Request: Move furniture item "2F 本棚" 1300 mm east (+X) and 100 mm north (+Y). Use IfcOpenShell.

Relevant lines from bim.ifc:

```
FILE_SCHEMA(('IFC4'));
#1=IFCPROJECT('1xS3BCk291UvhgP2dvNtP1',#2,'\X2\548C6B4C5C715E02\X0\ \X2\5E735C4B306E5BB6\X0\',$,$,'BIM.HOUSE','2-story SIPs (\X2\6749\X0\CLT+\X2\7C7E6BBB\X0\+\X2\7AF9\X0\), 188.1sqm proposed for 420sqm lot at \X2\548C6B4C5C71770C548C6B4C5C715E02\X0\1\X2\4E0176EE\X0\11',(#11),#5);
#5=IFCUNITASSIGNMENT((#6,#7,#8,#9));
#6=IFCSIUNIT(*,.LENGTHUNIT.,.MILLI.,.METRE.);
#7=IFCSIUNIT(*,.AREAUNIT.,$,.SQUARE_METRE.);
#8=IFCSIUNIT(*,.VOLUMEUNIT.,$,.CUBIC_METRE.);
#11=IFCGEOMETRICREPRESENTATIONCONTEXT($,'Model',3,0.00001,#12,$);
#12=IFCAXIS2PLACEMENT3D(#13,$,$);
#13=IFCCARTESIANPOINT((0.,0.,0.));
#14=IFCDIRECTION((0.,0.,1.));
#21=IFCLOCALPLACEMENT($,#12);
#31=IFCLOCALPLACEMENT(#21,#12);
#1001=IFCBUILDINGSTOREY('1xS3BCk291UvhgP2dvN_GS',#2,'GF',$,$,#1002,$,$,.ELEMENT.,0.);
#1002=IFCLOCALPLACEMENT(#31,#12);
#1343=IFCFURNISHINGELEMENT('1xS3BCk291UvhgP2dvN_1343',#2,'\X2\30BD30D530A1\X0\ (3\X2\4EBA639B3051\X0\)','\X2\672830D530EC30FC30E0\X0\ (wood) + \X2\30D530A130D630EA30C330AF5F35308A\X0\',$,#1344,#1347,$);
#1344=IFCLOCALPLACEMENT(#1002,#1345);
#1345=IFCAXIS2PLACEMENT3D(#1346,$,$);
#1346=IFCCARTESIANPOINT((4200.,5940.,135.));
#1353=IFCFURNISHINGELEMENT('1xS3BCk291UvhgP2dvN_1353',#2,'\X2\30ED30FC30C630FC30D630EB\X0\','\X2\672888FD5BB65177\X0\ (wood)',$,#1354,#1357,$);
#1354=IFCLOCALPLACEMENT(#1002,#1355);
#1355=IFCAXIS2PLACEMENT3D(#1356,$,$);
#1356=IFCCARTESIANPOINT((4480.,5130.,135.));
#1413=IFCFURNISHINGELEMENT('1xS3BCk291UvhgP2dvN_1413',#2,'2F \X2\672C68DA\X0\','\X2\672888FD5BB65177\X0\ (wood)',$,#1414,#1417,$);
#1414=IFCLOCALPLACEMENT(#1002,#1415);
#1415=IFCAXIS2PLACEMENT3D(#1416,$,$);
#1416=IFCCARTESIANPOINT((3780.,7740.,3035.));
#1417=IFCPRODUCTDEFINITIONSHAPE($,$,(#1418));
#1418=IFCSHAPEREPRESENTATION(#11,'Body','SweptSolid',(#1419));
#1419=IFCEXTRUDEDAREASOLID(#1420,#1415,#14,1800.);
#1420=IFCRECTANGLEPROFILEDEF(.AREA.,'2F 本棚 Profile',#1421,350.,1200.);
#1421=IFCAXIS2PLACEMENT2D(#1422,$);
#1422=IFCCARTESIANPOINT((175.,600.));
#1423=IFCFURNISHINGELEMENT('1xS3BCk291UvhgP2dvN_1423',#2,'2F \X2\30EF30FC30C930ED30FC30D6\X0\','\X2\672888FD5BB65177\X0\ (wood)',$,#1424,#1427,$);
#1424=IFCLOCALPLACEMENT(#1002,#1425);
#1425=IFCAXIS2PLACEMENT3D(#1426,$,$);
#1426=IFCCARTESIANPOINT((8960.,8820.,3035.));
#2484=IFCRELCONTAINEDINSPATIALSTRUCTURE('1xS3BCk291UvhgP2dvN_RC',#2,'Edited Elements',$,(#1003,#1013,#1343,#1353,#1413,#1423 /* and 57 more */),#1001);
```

```python
import ifcopenshell
import ifcopenshell.api.geometry
import ifcopenshell.util.placement
import ifcopenshell.util.unit

model = ifcopenshell.open("bim.ifc")
unit_scale = ifcopenshell.util.unit.calculate_unit_scale(model)

item = model.by_guid("1xS3BCk291UvhgP2dvN_1413")
matrix = ifcopenshell.util.placement.get_local_placement(item.ObjectPlacement)
matrix[0, 3] += 1.3 / unit_scale
matrix[1, 3] += 0.1 / unit_scale
ifcopenshell.api.geometry.edit_object_placement(model, product=item, matrix=matrix, is_si=False)

print(ifcopenshell.util.placement.get_local_placement(item.ObjectPlacement).round(3) + 0.0)

model.write("bim_v2.ifc")
```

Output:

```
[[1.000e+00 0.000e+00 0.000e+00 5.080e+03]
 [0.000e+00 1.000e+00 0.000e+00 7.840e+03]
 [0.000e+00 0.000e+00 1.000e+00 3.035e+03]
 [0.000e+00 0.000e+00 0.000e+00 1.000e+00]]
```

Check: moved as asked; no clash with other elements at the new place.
